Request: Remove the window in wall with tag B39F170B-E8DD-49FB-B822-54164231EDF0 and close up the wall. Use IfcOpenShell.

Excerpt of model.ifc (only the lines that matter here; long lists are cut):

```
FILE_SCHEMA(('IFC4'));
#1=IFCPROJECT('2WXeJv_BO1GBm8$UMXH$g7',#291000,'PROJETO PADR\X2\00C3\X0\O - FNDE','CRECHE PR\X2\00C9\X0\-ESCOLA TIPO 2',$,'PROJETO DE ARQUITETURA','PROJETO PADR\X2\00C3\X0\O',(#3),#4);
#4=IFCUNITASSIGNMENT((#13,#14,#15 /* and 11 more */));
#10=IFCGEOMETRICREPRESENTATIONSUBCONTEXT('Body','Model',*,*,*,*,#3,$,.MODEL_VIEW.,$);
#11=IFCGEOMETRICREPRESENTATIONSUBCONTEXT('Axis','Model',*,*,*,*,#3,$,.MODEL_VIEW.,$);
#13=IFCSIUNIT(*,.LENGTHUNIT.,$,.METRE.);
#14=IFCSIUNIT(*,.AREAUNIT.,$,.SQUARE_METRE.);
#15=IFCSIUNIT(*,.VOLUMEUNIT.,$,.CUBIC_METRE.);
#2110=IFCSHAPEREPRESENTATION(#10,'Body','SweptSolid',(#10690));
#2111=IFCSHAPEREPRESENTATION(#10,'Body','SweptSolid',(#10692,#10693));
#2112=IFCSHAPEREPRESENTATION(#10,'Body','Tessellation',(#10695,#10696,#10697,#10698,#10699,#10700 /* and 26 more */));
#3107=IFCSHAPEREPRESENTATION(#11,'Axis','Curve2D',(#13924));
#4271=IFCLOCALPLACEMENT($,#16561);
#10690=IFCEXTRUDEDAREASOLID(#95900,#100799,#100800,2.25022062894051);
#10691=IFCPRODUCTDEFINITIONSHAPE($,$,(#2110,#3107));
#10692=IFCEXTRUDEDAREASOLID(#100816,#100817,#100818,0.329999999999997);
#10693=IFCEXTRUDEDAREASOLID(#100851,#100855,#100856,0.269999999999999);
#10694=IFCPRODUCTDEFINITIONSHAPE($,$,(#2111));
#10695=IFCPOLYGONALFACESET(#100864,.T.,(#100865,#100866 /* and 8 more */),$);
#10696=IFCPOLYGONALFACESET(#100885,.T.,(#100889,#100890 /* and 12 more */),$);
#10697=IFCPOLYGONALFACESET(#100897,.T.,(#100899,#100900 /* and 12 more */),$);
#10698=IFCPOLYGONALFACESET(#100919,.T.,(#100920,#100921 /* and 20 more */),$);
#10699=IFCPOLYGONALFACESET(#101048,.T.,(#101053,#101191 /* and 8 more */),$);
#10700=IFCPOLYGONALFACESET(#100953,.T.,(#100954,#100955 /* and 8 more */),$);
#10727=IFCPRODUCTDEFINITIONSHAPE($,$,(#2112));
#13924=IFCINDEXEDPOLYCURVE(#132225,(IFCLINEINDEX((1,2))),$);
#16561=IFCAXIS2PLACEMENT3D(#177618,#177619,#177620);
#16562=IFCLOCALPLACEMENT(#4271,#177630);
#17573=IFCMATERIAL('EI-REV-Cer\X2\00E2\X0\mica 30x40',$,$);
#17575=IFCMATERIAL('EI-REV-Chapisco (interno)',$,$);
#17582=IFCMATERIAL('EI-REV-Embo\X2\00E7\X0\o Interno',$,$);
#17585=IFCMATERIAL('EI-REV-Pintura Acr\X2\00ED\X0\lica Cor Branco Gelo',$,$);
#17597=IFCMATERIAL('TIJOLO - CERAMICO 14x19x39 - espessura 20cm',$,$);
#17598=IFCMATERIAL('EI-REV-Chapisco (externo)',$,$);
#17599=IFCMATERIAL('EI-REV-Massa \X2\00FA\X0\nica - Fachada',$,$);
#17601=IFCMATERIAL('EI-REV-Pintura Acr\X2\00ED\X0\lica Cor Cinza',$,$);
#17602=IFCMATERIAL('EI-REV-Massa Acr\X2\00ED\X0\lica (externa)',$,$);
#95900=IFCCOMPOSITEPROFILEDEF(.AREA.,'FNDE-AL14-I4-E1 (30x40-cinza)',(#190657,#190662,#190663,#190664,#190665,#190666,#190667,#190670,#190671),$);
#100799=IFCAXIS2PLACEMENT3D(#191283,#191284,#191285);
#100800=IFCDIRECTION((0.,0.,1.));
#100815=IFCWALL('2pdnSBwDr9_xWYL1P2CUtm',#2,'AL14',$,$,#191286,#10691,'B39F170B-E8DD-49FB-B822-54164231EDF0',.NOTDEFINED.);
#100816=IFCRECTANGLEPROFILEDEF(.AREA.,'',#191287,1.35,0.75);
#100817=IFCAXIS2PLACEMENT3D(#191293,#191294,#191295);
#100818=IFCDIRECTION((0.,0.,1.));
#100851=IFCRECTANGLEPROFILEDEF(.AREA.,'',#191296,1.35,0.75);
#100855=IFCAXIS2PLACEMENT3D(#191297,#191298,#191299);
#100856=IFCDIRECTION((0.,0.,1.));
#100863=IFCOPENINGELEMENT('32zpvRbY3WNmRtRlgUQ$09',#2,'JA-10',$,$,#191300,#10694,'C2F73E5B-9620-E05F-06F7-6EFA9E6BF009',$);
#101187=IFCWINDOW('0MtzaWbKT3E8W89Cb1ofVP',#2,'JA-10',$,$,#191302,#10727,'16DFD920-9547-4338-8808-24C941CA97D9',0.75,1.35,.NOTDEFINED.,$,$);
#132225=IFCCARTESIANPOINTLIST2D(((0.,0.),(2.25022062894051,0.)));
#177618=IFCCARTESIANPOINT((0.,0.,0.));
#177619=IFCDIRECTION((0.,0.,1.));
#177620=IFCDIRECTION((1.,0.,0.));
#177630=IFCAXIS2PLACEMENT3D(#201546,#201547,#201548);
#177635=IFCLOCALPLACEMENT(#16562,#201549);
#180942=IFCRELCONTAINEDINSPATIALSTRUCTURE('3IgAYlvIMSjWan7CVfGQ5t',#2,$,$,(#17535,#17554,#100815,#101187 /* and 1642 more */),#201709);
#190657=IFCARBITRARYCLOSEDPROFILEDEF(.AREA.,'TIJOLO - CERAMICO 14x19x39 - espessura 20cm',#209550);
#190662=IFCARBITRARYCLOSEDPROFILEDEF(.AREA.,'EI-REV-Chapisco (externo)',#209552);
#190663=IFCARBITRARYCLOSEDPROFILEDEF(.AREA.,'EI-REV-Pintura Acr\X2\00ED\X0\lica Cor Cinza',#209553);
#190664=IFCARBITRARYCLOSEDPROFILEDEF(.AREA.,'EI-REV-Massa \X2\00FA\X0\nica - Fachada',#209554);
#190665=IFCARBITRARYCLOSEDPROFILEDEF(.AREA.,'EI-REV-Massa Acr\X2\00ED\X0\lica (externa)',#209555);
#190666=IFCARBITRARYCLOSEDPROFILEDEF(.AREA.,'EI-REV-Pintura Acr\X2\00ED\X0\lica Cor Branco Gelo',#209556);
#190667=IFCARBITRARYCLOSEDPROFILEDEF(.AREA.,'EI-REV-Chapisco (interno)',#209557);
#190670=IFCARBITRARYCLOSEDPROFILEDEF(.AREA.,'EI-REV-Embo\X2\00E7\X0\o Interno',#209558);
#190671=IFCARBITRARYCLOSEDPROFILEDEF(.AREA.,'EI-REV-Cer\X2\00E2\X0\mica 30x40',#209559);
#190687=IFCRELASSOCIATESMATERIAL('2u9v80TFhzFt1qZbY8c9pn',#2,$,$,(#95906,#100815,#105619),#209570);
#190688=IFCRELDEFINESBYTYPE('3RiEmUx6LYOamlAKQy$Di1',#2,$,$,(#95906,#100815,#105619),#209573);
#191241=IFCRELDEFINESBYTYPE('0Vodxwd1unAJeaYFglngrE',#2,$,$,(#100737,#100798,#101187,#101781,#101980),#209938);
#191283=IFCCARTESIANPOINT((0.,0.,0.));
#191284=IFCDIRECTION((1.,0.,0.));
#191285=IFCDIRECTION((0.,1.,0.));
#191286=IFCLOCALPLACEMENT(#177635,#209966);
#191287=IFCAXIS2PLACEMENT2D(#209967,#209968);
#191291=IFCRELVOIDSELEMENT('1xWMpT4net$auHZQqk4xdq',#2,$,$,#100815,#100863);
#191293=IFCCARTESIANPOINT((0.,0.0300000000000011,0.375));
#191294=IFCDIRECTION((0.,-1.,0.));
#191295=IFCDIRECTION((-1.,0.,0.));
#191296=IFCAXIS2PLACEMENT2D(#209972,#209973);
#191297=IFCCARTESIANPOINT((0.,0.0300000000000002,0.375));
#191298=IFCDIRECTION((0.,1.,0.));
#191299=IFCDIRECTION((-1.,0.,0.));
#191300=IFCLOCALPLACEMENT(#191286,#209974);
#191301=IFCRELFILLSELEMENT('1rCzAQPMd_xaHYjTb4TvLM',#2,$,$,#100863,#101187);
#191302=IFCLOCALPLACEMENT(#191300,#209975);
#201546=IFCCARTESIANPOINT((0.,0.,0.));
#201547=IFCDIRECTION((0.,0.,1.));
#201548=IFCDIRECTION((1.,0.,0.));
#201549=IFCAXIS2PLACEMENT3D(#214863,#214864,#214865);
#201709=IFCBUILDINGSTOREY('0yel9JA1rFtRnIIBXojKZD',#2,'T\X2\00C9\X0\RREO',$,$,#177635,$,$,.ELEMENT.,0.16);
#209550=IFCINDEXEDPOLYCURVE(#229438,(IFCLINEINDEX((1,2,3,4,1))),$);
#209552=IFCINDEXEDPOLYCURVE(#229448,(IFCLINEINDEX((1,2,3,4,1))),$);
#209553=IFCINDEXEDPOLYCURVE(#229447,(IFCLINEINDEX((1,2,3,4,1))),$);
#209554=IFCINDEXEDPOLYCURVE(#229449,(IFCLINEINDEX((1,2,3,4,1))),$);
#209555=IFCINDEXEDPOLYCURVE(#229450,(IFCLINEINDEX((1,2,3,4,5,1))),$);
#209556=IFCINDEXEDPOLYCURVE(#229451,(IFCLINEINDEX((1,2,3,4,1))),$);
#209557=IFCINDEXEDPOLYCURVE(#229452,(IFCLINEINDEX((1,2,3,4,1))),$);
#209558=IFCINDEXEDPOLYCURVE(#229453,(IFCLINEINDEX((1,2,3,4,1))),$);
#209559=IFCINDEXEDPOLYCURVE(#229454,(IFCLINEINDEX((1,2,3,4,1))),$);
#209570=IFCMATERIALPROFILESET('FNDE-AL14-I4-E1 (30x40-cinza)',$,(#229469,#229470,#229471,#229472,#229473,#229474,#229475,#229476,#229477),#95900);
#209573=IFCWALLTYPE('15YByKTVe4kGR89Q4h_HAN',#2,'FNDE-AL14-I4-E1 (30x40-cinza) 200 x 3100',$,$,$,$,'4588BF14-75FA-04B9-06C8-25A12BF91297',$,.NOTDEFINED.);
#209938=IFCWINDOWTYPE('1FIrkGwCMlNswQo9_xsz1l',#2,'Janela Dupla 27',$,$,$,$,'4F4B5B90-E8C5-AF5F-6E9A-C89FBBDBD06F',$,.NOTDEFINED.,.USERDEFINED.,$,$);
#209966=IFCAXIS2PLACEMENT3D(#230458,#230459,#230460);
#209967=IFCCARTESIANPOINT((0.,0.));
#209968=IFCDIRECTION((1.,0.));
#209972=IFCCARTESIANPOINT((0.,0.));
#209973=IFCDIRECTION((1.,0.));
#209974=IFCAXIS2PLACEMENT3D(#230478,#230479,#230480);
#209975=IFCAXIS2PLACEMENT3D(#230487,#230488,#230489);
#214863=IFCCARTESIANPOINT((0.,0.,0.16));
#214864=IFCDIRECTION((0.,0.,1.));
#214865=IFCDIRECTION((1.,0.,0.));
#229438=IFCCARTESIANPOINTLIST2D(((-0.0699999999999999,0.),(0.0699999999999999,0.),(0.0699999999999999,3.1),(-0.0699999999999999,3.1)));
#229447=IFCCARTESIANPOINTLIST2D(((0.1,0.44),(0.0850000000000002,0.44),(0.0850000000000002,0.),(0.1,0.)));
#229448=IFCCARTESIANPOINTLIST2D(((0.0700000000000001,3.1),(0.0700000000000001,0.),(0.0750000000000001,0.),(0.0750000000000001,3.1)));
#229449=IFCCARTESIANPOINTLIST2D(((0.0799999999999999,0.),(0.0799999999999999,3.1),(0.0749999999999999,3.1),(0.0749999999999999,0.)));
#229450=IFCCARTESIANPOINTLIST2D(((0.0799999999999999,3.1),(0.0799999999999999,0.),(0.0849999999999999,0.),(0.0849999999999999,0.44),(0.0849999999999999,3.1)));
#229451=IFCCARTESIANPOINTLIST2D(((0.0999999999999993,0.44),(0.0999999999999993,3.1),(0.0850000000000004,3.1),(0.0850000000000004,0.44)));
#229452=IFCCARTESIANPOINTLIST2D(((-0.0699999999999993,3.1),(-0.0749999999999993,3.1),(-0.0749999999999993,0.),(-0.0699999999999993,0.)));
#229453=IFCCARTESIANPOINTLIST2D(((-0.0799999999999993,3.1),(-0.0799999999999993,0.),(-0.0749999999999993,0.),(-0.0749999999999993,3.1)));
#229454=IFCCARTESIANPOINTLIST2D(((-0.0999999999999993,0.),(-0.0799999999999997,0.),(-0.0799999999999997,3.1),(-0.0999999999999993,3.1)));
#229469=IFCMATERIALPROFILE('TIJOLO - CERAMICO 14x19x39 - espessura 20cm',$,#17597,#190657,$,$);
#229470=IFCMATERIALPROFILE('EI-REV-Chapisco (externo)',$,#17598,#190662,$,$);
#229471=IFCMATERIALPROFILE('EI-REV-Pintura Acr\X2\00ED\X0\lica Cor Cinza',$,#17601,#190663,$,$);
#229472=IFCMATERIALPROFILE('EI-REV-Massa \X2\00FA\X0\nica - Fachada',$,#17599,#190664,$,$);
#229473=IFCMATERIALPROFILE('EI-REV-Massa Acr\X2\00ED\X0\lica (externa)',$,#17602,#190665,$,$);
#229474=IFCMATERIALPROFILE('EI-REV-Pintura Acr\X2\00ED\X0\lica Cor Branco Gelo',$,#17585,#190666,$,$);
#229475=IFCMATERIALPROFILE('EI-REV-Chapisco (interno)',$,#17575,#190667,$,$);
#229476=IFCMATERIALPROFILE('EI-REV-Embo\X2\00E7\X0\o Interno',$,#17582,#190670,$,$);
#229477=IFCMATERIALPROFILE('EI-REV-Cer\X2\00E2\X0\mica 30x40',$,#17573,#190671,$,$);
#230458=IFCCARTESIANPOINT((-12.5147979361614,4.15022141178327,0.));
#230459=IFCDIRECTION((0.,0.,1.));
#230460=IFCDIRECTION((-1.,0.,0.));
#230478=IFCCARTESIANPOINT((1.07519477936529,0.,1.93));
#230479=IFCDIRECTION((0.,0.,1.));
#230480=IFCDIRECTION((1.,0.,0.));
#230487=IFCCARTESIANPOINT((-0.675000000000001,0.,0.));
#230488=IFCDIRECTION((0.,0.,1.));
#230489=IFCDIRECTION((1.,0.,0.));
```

```python
import ifcopenshell
import ifcopenshell.api.feature
import ifcopenshell.api.root
import ifcopenshell.geom
import ifcopenshell.util.shape

model = ifcopenshell.open("model.ifc")
settings = ifcopenshell.geom.settings()


def volume(element):
    """Net volume in cubic metres, openings subtracted."""
    shape = ifcopenshell.geom.create_shape(settings, element)
    return ifcopenshell.util.shape.get_volume(shape.geometry)


window = model.by_guid("0MtzaWbKT3E8W89Cb1ofVP")
opening = window.FillsVoids[0].RelatingOpeningElement
wall = opening.VoidsElements[0].RelatingBuildingElement
before = volume(wall)

ifcopenshell.api.root.remove_product(model, product=window)
ifcopenshell.api.feature.remove_feature(model, feature=opening)

after = volume(wall)

print(f"wall volume {before:.3f} -> {after:.3f} m3")

model.write("model-out.ifc")
```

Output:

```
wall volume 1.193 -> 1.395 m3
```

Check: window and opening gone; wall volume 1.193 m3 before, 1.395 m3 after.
